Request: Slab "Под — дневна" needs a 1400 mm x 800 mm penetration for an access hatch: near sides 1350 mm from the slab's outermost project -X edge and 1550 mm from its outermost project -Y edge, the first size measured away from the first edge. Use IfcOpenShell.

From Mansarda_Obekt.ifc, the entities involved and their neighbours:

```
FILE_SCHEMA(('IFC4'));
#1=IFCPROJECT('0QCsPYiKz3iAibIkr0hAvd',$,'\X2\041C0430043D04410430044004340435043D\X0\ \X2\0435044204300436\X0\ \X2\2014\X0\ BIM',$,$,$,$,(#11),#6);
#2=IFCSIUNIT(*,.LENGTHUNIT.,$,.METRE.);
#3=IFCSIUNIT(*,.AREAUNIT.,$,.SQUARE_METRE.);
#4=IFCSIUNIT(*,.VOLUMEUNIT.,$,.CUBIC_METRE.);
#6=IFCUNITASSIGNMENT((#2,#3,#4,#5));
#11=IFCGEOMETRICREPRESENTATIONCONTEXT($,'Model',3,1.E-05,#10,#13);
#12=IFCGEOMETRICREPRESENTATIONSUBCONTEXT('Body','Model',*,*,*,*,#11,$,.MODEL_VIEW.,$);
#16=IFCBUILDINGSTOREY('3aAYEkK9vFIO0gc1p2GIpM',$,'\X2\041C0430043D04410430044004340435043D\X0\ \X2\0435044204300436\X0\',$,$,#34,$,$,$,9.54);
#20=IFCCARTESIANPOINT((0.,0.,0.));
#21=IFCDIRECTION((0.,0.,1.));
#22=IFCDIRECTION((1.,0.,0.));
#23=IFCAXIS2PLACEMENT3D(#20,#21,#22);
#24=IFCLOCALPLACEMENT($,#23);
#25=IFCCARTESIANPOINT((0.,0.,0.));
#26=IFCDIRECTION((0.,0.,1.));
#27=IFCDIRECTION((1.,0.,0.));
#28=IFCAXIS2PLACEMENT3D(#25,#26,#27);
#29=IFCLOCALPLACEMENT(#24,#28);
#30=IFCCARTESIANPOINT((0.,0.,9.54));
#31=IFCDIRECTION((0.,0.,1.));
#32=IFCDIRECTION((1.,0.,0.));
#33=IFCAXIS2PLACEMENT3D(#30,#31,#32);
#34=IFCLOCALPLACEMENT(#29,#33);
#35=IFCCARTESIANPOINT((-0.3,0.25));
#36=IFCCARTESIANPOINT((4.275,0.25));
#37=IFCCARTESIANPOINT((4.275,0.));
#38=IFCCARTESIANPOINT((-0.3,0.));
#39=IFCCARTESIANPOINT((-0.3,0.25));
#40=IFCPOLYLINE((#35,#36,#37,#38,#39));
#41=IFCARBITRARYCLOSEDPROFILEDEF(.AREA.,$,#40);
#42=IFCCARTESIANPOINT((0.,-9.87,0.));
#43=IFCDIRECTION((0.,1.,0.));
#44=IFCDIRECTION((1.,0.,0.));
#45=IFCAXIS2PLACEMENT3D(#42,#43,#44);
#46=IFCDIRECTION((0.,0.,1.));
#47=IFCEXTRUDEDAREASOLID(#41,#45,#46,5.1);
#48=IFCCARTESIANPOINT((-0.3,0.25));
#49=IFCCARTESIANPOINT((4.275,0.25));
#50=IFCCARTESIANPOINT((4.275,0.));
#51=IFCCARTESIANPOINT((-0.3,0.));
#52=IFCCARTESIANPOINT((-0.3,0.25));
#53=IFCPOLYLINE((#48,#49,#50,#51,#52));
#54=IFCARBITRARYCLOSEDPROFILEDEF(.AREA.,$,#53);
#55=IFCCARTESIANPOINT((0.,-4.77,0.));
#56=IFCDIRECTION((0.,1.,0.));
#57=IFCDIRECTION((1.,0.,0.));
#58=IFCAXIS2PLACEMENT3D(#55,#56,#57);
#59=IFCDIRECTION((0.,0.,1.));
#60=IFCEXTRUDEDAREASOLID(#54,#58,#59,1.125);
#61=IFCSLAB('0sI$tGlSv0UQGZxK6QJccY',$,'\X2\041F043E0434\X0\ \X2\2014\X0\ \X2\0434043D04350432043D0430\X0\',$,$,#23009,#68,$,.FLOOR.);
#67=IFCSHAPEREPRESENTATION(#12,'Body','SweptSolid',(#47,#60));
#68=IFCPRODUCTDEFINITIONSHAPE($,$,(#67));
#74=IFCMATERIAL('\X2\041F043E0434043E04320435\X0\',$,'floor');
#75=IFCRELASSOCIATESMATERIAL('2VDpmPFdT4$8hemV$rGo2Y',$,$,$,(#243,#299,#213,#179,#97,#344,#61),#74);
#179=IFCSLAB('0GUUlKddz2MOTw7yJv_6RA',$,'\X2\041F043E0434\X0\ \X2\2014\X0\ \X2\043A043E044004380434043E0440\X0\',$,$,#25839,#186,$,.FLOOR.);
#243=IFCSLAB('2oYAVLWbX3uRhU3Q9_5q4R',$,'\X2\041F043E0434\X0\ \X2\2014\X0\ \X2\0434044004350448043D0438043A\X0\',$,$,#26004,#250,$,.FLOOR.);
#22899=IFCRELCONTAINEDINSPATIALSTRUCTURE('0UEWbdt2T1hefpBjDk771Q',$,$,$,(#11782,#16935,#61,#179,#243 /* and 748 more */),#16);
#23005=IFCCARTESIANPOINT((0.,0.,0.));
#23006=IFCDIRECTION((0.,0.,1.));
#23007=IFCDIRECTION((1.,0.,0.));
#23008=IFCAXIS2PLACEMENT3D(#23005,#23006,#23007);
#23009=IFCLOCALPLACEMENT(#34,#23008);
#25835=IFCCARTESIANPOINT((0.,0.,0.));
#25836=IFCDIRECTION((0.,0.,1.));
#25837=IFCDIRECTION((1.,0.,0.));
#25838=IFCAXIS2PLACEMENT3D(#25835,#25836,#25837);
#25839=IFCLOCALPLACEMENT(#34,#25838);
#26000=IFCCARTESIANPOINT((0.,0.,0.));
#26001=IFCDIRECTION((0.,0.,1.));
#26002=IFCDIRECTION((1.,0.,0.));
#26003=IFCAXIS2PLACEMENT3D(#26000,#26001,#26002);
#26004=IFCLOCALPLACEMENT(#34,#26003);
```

```python
import numpy as np
import ifcopenshell
import ifcopenshell.api.feature
import ifcopenshell.api.geometry
import ifcopenshell.api.root
import ifcopenshell.geom
import ifcopenshell.util.placement
import ifcopenshell.util.representation
import ifcopenshell.util.shape
import ifcopenshell.util.unit

model = ifcopenshell.open("Mansarda_Obekt.ifc")
unit_scale = ifcopenshell.util.unit.calculate_unit_scale(model)
settings = ifcopenshell.geom.settings()


def volume(element):
    """Net volume in cubic metres, openings subtracted."""
    shape = ifcopenshell.geom.create_shape(settings, element)
    return ifcopenshell.util.shape.get_volume(shape.geometry)


slab = model.by_id(61)
before = volume(slab)

# Extent in the slab's own axes, in metres. The edges named are its -X and -Y sides.
slab_shape = ifcopenshell.geom.create_shape(settings, slab)
vertices = ifcopenshell.util.shape.get_vertices(slab_shape.geometry)
x_min, y_min, bottom = vertices.min(axis=0)
top = vertices[:, 2].max()

opening = ifcopenshell.api.root.create_entity(model, ifc_class="IfcOpeningElement", name="Access hatch opening", predefined_type="OPENING")
context = ifcopenshell.util.representation.get_context(model, "Model", "Body", "MODEL_VIEW")
width, depth = 1.4, 0.8
outline = [(0.0, 0.0), (width, 0.0), (width, depth), (0.0, depth), (0.0, 0.0)]
# Overshoot both faces by 50 mm so the cut is clean.
shape = ifcopenshell.api.geometry.add_slab_representation(
    model, context=context, depth=top - bottom + 0.1, polyline=outline
)
ifcopenshell.api.geometry.assign_representation(model, product=opening, representation=shape)

matrix = ifcopenshell.util.placement.get_local_placement(slab.ObjectPlacement)
matrix[:, 3] = matrix @ np.append(np.array([x_min + 1.35, y_min + 1.55, bottom - 0.05]) / unit_scale, 1.0)
ifcopenshell.api.geometry.edit_object_placement(model, product=opening, matrix=matrix, is_si=False)
ifcopenshell.api.feature.add_feature(model, feature=opening, element=slab)

after = volume(slab)

print(f"slab volume {before:.3f} -> {after:.3f} m3")

model.write("Mansarda_Obekt_rev.ifc")
```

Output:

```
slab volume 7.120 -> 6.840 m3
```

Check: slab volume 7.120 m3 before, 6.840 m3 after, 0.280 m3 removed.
